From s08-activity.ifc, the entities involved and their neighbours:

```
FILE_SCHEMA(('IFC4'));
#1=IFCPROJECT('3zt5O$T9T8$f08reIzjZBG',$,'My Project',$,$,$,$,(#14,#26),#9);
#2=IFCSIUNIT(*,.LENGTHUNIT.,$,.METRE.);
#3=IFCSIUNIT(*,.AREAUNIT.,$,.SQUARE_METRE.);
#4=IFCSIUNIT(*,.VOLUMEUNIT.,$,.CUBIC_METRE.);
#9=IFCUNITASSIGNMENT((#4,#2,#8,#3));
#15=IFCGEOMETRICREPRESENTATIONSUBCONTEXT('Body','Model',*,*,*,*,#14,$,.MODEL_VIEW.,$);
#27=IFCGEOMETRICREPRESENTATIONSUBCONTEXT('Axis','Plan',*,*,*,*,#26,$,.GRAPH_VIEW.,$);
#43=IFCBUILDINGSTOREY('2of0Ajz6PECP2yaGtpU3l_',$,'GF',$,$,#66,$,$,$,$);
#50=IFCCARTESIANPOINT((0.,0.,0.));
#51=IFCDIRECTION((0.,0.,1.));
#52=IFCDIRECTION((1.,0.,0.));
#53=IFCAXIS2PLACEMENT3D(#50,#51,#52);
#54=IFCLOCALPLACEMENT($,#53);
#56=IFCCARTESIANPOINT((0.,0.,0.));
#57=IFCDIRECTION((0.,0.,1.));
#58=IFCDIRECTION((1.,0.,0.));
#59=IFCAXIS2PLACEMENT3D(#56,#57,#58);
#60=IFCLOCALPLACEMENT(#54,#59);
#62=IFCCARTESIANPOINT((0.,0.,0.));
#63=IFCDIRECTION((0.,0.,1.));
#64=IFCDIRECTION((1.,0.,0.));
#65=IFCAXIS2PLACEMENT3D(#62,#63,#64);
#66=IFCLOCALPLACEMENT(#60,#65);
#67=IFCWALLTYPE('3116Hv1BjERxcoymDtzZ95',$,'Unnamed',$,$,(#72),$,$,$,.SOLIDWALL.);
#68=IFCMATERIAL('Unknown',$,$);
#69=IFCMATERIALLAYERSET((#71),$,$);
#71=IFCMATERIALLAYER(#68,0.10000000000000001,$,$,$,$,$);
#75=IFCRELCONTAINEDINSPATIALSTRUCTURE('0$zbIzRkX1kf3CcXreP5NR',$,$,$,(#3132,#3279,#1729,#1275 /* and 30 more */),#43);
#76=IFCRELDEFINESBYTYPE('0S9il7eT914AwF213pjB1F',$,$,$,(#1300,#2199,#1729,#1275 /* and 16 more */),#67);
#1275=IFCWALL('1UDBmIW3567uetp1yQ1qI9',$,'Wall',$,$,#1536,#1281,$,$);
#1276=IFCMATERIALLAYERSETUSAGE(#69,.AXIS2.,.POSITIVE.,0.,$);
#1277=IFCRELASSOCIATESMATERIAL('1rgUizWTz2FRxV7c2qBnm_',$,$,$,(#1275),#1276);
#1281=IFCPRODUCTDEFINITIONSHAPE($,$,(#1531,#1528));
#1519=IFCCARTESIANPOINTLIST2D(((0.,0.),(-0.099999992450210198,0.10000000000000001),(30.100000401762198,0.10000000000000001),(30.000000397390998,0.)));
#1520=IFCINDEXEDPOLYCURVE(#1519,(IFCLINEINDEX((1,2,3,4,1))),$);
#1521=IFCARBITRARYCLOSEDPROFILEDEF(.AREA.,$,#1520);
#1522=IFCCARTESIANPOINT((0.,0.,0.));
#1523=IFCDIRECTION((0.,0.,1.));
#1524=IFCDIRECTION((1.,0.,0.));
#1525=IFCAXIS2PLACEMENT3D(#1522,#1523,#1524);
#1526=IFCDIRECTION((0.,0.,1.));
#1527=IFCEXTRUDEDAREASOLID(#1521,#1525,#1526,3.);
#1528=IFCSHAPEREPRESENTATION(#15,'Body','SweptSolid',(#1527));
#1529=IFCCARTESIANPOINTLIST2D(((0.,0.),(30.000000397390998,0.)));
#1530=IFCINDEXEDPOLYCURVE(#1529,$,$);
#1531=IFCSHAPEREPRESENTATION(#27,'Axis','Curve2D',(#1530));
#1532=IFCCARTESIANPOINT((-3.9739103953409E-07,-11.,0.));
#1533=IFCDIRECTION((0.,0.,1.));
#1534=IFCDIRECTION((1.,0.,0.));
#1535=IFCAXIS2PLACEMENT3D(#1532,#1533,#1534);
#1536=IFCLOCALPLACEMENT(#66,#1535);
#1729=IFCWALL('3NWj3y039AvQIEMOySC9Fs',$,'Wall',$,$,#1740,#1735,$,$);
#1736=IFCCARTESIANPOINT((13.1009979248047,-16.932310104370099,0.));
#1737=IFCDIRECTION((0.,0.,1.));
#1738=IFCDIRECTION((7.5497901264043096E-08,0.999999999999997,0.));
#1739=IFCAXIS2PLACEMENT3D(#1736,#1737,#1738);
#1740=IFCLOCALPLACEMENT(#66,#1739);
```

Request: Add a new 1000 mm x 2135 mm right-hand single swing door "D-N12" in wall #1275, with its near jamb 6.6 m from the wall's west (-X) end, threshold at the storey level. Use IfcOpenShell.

```python
import numpy as np
import ifcopenshell
import ifcopenshell.api.feature
import ifcopenshell.api.geometry
import ifcopenshell.api.root
import ifcopenshell.api.spatial
import ifcopenshell.geom
import ifcopenshell.util.element
import ifcopenshell.util.placement
import ifcopenshell.util.representation
import ifcopenshell.util.shape
import ifcopenshell.util.unit

model = ifcopenshell.open("s08-activity.ifc")
unit_scale = ifcopenshell.util.unit.calculate_unit_scale(model)
settings = ifcopenshell.geom.settings()


def volume(element):
    """Net volume in cubic metres, openings subtracted."""
    shape = ifcopenshell.geom.create_shape(settings, element)
    return ifcopenshell.util.shape.get_volume(shape.geometry)


wall = model.by_id(1275)
storey = ifcopenshell.util.element.get_container(wall, ifc_class="IfcBuildingStorey")
context = ifcopenshell.util.representation.get_context(model, "Model", "Body", "MODEL_VIEW")
before = volume(wall)

width, height, from_end, sill = 1, 2.135, 6.6, 0.0  # metres

# The wall runs along its own X axis, and the end named is its -X end.
wall_shape = ifcopenshell.geom.create_shape(settings, wall)
x, y, z = ifcopenshell.util.shape.get_vertices(wall_shape.geometry).T
start = x.min() + from_end
face, thickness = float(y.min()), float(y.max() - y.min())
wall_matrix = ifcopenshell.util.placement.get_local_placement(wall.ObjectPlacement)
level = ifcopenshell.util.placement.get_local_placement(storey.ObjectPlacement)[2, 3]


def in_wall(x, y):
    """Placement at x, y metres in the wall's axes, at sill height."""
    matrix = wall_matrix.copy()
    matrix[:, 3] = wall_matrix @ np.array([x / unit_scale, y / unit_scale, 0.0, 1.0])
    matrix[2, 3] = level + sill / unit_scale
    return matrix


# Opening: a box that overshoots both wall faces by 50 mm.
opening = ifcopenshell.api.root.create_entity(model, ifc_class="IfcOpeningElement", predefined_type="OPENING")
box = ifcopenshell.api.geometry.add_wall_representation(
    model, context=context, length=width, height=height, thickness=thickness + 0.1
)
ifcopenshell.api.geometry.assign_representation(model, product=opening, representation=box)
ifcopenshell.api.geometry.edit_object_placement(model, product=opening, matrix=in_wall(start, face - 0.05), is_si=False)
ifcopenshell.api.feature.add_feature(model, feature=opening, element=wall)

door = ifcopenshell.api.root.create_entity(model, ifc_class="IfcDoor", name="D-N12", predefined_type="DOOR")
door.OverallWidth, door.OverallHeight = width / unit_scale, height / unit_scale
door.OperationType = "SINGLE_SWING_RIGHT"
body = ifcopenshell.api.geometry.add_door_representation(
    model,
    context=context,
    overall_width=door.OverallWidth,
    overall_height=door.OverallHeight,
    operation_type="SINGLE_SWING_RIGHT",
    lining_properties={"LiningDepth": thickness / unit_scale, "ThresholdDepth": thickness / unit_scale},
)
ifcopenshell.api.geometry.assign_representation(model, product=door, representation=body)
ifcopenshell.api.spatial.assign_container(model, products=[door], relating_structure=storey)
ifcopenshell.api.feature.add_filling(model, opening=opening, element=door)

# The lining spans the wall, so the door starts at the wall face.
ifcopenshell.api.geometry.edit_object_placement(model, product=door, matrix=in_wall(start, face), is_si=False)

after = volume(wall)

print(f"wall volume {before:.3f} -> {after:.3f} m3")

model.write("s08-activity_rev.ifc")
```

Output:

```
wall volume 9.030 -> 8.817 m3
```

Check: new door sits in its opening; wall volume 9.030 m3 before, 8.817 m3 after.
